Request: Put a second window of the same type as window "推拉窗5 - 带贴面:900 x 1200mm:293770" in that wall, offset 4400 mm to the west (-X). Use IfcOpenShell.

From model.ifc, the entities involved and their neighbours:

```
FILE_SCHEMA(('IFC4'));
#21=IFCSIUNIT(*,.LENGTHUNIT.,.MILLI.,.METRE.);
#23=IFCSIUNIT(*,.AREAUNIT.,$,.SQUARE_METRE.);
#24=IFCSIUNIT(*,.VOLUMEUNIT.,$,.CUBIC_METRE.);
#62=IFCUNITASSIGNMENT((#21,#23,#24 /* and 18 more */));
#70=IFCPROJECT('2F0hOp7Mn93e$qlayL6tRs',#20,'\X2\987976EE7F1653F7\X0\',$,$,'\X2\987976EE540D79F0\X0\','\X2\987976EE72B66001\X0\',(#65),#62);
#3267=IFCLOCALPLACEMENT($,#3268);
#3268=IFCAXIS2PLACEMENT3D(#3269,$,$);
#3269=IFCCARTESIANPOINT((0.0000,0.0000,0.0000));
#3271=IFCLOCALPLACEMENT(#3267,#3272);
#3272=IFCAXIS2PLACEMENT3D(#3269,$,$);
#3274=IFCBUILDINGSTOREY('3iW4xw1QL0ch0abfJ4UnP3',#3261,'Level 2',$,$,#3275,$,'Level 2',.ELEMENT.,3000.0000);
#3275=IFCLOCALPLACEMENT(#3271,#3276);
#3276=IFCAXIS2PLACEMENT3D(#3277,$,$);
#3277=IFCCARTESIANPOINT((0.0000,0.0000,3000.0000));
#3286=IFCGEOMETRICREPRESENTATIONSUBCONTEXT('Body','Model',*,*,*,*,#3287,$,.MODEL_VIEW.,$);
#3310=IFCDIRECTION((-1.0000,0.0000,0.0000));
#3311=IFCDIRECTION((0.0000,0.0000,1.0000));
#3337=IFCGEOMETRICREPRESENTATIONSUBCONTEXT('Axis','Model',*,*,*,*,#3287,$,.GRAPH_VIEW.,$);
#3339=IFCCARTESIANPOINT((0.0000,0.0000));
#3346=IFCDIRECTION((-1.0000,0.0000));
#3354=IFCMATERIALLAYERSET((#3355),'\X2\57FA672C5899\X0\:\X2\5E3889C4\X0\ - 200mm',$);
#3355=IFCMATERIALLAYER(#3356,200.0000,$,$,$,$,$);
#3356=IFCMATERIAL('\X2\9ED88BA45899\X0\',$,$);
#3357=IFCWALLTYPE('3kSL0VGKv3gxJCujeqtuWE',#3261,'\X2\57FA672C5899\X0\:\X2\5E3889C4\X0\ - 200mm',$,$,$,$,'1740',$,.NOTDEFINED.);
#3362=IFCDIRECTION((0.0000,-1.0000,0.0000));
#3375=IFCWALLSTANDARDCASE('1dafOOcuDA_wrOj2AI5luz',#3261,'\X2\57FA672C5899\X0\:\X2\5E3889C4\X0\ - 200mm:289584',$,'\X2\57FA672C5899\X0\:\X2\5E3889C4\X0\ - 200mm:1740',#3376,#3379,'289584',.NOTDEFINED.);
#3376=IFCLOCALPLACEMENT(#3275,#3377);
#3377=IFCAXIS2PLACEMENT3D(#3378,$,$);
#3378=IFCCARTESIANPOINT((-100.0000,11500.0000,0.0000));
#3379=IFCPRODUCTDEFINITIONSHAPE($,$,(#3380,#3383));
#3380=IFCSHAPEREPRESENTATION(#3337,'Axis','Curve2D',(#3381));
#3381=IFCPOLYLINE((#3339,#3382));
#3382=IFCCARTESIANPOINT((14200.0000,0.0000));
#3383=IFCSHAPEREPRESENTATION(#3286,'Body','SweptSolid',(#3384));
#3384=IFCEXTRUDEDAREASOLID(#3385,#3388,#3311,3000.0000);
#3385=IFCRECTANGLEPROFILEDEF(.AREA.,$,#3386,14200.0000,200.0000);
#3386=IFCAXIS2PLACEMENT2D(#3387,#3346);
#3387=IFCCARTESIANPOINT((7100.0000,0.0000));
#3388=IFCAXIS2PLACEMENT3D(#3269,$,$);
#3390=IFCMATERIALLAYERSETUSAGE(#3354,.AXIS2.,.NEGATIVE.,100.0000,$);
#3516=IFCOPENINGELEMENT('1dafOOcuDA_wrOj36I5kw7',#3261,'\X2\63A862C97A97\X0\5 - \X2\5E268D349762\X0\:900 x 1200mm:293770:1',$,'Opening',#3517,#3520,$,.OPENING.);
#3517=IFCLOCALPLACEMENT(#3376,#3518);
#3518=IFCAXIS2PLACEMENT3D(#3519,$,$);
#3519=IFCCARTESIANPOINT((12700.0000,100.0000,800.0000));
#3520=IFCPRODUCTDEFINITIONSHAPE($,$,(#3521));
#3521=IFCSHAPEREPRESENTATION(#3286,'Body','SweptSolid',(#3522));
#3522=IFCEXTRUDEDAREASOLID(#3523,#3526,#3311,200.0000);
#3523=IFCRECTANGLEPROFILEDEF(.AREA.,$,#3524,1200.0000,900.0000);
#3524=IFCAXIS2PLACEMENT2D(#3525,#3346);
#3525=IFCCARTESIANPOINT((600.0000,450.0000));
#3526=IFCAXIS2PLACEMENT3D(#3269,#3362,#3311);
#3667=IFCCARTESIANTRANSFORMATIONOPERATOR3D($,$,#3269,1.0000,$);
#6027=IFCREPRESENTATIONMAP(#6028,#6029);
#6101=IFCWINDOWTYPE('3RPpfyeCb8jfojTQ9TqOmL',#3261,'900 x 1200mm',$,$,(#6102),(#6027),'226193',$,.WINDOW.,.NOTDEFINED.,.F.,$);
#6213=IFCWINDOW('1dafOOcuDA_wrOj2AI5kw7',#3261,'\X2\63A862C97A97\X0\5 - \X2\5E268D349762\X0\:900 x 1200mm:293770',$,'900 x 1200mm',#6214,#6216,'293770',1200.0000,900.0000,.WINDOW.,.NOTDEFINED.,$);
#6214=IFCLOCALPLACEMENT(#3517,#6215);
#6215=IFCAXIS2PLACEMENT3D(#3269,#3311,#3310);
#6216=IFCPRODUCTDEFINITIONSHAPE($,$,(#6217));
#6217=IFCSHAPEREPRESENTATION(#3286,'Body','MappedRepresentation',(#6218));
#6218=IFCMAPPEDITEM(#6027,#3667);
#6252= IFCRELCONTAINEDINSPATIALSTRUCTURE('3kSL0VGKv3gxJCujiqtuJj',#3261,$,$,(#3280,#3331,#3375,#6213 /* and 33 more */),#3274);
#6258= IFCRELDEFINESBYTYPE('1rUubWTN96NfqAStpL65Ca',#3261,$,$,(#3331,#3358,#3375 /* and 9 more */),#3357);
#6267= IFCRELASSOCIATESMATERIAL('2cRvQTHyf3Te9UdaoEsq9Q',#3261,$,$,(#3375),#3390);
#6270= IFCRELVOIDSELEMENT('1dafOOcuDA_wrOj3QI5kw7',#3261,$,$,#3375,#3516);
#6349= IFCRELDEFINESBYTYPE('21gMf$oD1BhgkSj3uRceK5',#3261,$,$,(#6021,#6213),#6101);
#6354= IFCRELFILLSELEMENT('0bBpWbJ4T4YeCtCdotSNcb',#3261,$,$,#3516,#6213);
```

```python
import ifcopenshell
import ifcopenshell.api.feature
import ifcopenshell.api.geometry
import ifcopenshell.api.root
import ifcopenshell.geom
import ifcopenshell.util.element
import ifcopenshell.util.placement
import ifcopenshell.util.shape

model = ifcopenshell.open("model.ifc")
settings = ifcopenshell.geom.settings()


def volume(element):
    """Net volume in cubic metres, openings subtracted."""
    shape = ifcopenshell.geom.create_shape(settings, element)
    return ifcopenshell.util.shape.get_volume(shape.geometry)


def reuse_history(source, copy):
    """copy_class also copies each property set's owner history, people and application; keep the originals."""
    for rel in copy.IsDefinedBy:
        if rel.is_a("IfcRelDefinesByProperties") and (history := rel.RelatingPropertyDefinition.OwnerHistory):
            rel.RelatingPropertyDefinition.OwnerHistory = source.OwnerHistory
            ifcopenshell.util.element.remove_deep2(model, history)


window = model.by_id(6213)
opening = window.FillsVoids[0].RelatingOpeningElement
wall = opening.VoidsElements[0].RelatingBuildingElement
before = volume(wall)
shift = ifcopenshell.util.placement.get_local_placement(wall.ObjectPlacement)[:3, 0] * -4400.0

# copy_class copies the void relationship, type, container and properties, but no geometry.
new_opening = ifcopenshell.api.root.copy_class(model, product=opening)
new_opening.Representation = ifcopenshell.util.element.copy_deep(
    model, opening.Representation, exclude=["IfcGeometricRepresentationContext", "IfcRepresentationMap"]
)
new_opening.Name = "推拉窗5 - 带贴面:900 x 1200mm"
new_window = ifcopenshell.api.root.copy_class(model, product=window)
new_window.Representation = ifcopenshell.util.element.copy_deep(
    model, window.Representation, exclude=["IfcGeometricRepresentationContext", "IfcRepresentationMap"]
)
new_window.Name = "推拉窗5 - 带贴面:900 x 1200mm"
new_window.Tag = None
reuse_history(window, new_window)
ifcopenshell.api.feature.add_filling(model, opening=new_opening, element=new_window)

for old, new in ((opening, new_opening), (window, new_window)):
    matrix = ifcopenshell.util.placement.get_local_placement(old.ObjectPlacement)
    matrix[:3, 3] += shift
    ifcopenshell.api.geometry.edit_object_placement(model, product=new, matrix=matrix, is_si=False)

after = volume(wall)

print(f"wall volume {before:.3f} -> {after:.3f} m3")

model.write("model_v2.ifc")
```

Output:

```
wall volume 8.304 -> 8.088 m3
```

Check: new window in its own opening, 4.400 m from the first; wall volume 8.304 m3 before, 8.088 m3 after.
